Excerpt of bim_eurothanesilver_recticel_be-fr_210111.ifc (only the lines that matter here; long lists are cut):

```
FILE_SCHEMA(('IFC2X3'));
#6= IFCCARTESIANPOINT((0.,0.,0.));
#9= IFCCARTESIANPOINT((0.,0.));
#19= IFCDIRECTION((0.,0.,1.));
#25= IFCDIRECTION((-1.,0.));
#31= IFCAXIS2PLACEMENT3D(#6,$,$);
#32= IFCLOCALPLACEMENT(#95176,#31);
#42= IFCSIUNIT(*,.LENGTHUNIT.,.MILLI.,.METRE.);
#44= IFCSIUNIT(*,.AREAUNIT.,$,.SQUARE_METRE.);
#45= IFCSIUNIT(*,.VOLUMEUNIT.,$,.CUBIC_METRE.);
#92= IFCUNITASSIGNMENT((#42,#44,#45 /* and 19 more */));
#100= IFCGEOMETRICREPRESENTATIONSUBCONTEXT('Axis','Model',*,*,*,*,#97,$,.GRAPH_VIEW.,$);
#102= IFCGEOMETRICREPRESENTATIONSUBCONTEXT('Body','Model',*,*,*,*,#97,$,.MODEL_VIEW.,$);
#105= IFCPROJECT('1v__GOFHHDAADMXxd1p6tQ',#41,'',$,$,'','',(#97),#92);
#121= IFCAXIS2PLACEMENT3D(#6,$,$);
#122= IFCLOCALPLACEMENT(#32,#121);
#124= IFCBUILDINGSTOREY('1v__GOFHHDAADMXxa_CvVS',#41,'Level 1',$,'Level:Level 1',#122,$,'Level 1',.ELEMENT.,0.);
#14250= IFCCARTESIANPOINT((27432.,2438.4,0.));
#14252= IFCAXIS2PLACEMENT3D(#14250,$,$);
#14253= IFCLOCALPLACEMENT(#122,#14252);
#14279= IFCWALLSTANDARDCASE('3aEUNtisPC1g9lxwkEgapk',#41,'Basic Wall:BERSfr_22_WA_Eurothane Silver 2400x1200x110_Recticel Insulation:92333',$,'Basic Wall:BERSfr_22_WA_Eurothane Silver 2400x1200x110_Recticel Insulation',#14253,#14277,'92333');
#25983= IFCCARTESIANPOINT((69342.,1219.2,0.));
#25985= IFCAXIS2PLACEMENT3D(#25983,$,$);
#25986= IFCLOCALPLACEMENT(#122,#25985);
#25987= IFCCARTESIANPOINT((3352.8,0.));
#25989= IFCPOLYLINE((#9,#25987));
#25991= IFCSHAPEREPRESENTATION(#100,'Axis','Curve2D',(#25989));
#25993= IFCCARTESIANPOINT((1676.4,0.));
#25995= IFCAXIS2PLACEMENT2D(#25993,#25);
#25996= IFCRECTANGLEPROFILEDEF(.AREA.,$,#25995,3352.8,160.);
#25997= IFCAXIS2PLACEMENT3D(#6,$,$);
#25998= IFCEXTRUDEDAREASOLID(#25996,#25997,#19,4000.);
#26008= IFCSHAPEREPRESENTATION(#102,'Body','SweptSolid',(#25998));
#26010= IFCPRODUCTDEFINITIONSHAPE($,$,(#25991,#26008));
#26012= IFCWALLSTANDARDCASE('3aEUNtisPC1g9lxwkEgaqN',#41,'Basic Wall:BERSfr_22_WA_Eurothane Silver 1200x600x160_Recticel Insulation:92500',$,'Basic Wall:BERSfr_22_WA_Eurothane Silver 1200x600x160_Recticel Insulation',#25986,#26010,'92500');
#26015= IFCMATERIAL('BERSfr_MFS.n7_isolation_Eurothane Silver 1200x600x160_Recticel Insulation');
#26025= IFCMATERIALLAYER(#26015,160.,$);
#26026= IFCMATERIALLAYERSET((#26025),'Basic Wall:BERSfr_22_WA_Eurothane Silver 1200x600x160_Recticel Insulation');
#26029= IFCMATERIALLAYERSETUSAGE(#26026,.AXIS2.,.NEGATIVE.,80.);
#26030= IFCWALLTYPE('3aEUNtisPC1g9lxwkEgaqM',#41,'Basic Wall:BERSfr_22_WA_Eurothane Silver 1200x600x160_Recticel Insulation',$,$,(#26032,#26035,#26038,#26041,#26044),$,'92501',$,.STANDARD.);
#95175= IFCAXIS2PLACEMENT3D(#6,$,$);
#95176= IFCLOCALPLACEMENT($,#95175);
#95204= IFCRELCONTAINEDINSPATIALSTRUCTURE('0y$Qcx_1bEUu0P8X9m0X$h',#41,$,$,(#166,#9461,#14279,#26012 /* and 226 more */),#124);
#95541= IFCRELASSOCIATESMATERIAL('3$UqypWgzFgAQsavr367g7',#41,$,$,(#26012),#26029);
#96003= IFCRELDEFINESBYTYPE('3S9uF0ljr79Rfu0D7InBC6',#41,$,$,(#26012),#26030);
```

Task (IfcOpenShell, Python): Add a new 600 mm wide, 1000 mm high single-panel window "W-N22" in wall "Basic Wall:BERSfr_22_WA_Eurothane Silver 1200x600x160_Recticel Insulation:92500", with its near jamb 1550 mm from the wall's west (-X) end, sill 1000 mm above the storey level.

```python
import numpy as np
import ifcopenshell
import ifcopenshell.api.feature
import ifcopenshell.api.geometry
import ifcopenshell.api.root
import ifcopenshell.api.spatial
import ifcopenshell.api.type
import ifcopenshell.geom
import ifcopenshell.util.element
import ifcopenshell.util.placement
import ifcopenshell.util.representation
import ifcopenshell.util.shape
import ifcopenshell.util.unit

model = ifcopenshell.open("bim_eurothanesilver_recticel_be-fr_210111.ifc")
unit_scale = ifcopenshell.util.unit.calculate_unit_scale(model)
settings = ifcopenshell.geom.settings()


def volume(element):
    """Net volume in cubic metres, openings subtracted."""
    shape = ifcopenshell.geom.create_shape(settings, element)
    return ifcopenshell.util.shape.get_volume(shape.geometry)


wall = model.by_id(26012)
storey = ifcopenshell.util.element.get_container(wall, ifc_class="IfcBuildingStorey")
context = ifcopenshell.util.representation.get_context(model, "Model", "Body", "MODEL_VIEW")
before = volume(wall)

width, height, from_end, sill = 0.6, 1, 1.55, 1  # metres

# The wall runs along its own X axis, and the end named is its -X end.
wall_shape = ifcopenshell.geom.create_shape(settings, wall)
x, y, z = ifcopenshell.util.shape.get_vertices(wall_shape.geometry).T
start = x.min() + from_end
face, thickness = float(y.min()), float(y.max() - y.min())
wall_matrix = ifcopenshell.util.placement.get_local_placement(wall.ObjectPlacement)
level = ifcopenshell.util.placement.get_local_placement(storey.ObjectPlacement)[2, 3]


def in_wall(x, y):
    """Placement at x, y metres in the wall's axes, at sill height."""
    matrix = wall_matrix.copy()
    matrix[:, 3] = wall_matrix @ np.array([x / unit_scale, y / unit_scale, 0.0, 1.0])
    matrix[2, 3] = level + sill / unit_scale
    return matrix


# Opening: a box that overshoots both wall faces by 50 mm.
opening = ifcopenshell.api.root.create_entity(model, ifc_class="IfcOpeningElement")
box = ifcopenshell.api.geometry.add_wall_representation(
    model, context=context, length=width, height=height, thickness=thickness + 0.1
)
ifcopenshell.api.geometry.assign_representation(model, product=opening, representation=box)
ifcopenshell.api.geometry.edit_object_placement(model, product=opening, matrix=in_wall(start, face - 0.05), is_si=False)
ifcopenshell.api.feature.add_feature(model, feature=opening, element=wall)

window = ifcopenshell.api.root.create_entity(model, ifc_class="IfcWindow", name="W-N22")
window.OverallWidth, window.OverallHeight = width / unit_scale, height / unit_scale
body = ifcopenshell.api.geometry.add_window_representation(
    model,
    context=context,
    overall_width=window.OverallWidth,
    overall_height=window.OverallHeight,
    partition_type="SINGLE_PANEL",
)
ifcopenshell.api.geometry.assign_representation(model, product=window, representation=body)
ifcopenshell.api.spatial.assign_container(model, products=[window], relating_structure=storey)
fills = ifcopenshell.api.feature.add_filling(model, opening=opening, element=window)
fills.OwnerHistory = window.OwnerHistory  # required in IFC2X3

# IFC2X3 keeps the operation on the window style.
style = ifcopenshell.api.root.create_entity(model, ifc_class="IfcWindowStyle", name="W-N22")
style.OperationType, style.ConstructionType = "SINGLE_PANEL", "NOTDEFINED"
style.ParameterTakesPrecedence = style.Sizeable = False
ifcopenshell.api.type.assign_type(model, related_objects=[window], relating_type=style)

# Centre the window in the wall's thickness.
ifcopenshell.api.geometry.edit_object_placement(model, product=window, matrix=in_wall(start, face), is_si=False)
window_shape = ifcopenshell.geom.create_shape(settings, window)
depth = ifcopenshell.util.shape.get_vertices(window_shape.geometry)[:, 1]
offset = face + thickness / 2 - (depth.min() + depth.max()) / 2
ifcopenshell.api.geometry.edit_object_placement(model, product=window, matrix=in_wall(start, offset), is_si=False)

after = volume(wall)

print(f"wall volume {before:.3f} -> {after:.3f} m3")

model.write("bim_eurothanesilver_recticel_be-fr_210111_updated.ifc")
```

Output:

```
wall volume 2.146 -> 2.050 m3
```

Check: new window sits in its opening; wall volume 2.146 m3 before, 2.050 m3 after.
